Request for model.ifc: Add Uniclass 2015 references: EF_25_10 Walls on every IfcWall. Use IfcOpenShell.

First a look at what the model holds.

```python
import ifcopenshell

model = ifcopenshell.open("model.ifc")
print(model.schema)
print("classifications:", [c.Name for c in model.by_type("IfcClassification")])
for ifc_class in ("IfcDoor", "IfcRoof", "IfcStair", "IfcWall", "IfcWindow"):
    print(ifc_class, len(model.by_type(ifc_class)))
```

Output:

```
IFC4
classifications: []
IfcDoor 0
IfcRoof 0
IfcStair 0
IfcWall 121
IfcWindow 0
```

```python
import ifcopenshell
import ifcopenshell.api.classification

model = ifcopenshell.open("model.ifc")

system = ifcopenshell.api.classification.add_classification(model, classification="Uniclass 2015")

codes = {
    "IfcWall": ("EF_25_10", "Walls"),
}
for ifc_class, (code, name) in codes.items():
    products = model.by_type(ifc_class)
    ifcopenshell.api.classification.add_reference(
        model, products=products, classification=system, identification=code, name=name
    )
    print(code, len(products))

model.write("model_rev.ifc")
```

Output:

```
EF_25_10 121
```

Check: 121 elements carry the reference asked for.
